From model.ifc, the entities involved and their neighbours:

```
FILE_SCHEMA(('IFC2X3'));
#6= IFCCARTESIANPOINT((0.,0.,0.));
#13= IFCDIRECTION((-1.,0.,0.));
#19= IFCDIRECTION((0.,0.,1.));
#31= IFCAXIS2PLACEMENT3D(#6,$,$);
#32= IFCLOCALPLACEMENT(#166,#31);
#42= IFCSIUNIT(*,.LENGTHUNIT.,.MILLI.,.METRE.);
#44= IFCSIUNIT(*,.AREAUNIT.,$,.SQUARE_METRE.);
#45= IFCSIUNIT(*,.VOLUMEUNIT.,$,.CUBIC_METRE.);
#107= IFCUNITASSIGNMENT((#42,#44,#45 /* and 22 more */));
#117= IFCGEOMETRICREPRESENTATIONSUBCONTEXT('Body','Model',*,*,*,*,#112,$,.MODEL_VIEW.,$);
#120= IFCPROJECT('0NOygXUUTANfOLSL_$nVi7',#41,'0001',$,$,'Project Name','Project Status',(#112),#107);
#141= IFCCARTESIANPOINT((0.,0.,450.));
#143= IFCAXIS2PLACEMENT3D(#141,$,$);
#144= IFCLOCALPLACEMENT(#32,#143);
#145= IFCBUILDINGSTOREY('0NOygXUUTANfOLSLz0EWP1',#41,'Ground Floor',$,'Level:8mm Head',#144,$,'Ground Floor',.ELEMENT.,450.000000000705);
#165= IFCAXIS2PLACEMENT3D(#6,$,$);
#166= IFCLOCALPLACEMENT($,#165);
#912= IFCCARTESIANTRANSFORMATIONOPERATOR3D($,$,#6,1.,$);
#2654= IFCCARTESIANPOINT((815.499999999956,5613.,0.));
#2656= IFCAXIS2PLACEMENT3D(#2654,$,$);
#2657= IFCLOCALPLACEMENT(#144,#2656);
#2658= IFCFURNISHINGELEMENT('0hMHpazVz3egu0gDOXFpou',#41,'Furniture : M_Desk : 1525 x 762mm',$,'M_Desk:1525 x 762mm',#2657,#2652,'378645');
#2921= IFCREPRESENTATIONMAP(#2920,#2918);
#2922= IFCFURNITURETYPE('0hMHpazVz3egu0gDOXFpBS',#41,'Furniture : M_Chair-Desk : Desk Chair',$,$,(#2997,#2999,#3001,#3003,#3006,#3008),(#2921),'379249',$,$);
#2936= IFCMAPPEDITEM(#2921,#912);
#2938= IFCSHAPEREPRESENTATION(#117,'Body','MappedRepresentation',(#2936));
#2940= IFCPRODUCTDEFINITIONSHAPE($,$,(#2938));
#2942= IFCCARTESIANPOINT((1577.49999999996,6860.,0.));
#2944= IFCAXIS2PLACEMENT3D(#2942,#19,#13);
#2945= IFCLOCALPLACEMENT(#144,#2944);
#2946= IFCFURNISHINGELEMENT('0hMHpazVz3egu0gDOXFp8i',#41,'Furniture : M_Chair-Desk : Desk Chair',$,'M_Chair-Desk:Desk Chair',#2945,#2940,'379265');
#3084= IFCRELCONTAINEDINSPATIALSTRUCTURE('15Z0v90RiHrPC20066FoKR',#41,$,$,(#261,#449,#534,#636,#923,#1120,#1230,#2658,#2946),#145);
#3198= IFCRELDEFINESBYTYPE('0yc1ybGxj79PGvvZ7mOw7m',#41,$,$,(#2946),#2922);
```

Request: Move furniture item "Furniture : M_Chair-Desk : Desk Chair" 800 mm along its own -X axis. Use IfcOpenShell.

```python
import ifcopenshell
import ifcopenshell.api.geometry
import ifcopenshell.util.placement
import ifcopenshell.util.unit

model = ifcopenshell.open("model.ifc")
unit_scale = ifcopenshell.util.unit.calculate_unit_scale(model)

item = model.by_guid("0hMHpazVz3egu0gDOXFp8i")
matrix = ifcopenshell.util.placement.get_local_placement(item.ObjectPlacement)
matrix[:3, 3] -= matrix[:3, 0] * 0.8 / unit_scale
ifcopenshell.api.geometry.edit_object_placement(model, product=item, matrix=matrix, is_si=False)

print(ifcopenshell.util.placement.get_local_placement(item.ObjectPlacement).round(3) + 0.0)

model.write("model_edited.ifc")
```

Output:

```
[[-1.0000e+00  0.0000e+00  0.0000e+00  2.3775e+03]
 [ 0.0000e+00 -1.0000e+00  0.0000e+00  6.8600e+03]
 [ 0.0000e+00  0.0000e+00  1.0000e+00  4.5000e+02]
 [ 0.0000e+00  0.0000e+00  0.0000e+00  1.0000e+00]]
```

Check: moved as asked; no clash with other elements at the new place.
